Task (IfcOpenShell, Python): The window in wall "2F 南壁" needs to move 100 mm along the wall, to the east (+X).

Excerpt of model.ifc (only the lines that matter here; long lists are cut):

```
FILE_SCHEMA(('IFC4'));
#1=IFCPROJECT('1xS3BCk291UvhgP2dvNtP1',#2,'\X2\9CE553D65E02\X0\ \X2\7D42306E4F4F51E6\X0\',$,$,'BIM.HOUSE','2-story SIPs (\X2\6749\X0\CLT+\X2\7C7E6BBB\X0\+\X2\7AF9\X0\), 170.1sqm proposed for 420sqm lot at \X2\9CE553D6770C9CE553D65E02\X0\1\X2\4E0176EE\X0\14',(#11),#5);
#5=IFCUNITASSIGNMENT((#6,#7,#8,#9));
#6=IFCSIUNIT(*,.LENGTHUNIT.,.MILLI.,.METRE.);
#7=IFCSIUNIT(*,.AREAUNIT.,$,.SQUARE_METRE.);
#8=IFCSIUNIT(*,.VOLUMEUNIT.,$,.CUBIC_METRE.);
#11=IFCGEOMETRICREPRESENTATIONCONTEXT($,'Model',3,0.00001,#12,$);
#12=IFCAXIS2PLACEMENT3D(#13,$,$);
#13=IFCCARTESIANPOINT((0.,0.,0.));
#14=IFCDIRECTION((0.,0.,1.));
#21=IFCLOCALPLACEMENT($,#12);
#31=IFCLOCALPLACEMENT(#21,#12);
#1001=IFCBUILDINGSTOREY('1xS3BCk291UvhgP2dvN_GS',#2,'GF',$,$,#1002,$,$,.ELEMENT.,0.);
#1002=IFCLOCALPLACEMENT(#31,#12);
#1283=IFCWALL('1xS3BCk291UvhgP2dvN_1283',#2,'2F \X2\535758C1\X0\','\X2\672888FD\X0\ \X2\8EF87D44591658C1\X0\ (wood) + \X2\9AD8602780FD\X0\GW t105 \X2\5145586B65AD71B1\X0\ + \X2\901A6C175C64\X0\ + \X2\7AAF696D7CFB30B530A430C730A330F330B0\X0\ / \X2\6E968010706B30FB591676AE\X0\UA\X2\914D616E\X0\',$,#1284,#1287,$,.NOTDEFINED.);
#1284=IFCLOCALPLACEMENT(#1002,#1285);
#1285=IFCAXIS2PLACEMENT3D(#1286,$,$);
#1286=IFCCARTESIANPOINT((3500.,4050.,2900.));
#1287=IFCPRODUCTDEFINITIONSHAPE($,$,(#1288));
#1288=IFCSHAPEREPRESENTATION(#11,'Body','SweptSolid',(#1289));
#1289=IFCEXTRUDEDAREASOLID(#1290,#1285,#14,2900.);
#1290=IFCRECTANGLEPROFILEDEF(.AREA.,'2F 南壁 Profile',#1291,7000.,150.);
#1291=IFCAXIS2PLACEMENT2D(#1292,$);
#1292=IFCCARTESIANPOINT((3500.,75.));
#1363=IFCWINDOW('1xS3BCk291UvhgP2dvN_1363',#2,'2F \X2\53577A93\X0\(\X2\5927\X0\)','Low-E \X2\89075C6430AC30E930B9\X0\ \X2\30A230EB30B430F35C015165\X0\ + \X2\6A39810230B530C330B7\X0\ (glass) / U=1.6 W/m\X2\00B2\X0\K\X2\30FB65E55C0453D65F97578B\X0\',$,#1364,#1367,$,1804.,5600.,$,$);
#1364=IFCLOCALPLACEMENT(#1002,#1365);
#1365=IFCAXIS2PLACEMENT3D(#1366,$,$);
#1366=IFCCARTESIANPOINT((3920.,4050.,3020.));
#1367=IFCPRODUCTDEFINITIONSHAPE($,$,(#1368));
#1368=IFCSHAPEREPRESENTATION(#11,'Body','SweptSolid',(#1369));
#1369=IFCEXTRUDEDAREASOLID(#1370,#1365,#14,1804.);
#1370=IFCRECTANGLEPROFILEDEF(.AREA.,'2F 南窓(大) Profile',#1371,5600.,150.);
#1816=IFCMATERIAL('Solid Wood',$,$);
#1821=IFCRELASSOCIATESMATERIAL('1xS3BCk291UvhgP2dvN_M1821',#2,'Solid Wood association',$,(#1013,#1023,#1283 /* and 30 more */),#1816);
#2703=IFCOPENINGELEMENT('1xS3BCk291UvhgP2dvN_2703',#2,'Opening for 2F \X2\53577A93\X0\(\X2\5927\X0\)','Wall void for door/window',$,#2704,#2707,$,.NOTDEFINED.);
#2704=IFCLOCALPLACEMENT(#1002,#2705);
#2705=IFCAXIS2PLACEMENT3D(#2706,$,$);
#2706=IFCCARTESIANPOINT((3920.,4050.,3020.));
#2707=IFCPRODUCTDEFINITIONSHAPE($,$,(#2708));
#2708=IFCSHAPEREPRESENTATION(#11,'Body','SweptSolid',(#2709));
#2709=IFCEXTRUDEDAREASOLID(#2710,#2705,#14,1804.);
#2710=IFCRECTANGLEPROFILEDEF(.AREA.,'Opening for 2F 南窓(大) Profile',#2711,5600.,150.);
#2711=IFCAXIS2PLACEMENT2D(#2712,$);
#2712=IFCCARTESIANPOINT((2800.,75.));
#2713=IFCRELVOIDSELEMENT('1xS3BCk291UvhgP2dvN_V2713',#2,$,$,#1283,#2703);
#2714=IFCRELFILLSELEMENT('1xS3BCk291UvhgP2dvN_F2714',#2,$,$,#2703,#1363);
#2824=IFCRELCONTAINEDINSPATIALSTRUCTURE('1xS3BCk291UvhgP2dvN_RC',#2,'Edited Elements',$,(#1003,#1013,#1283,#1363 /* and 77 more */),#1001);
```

```python
import ifcopenshell
import ifcopenshell.api.geometry
import ifcopenshell.util.placement
import ifcopenshell.util.unit

model = ifcopenshell.open("model.ifc")
unit_scale = ifcopenshell.util.unit.calculate_unit_scale(model)

window = model.by_guid("1xS3BCk291UvhgP2dvN_1363")
opening = window.FillsVoids[0].RelatingOpeningElement
wall = opening.VoidsElements[0].RelatingBuildingElement

wall_matrix = ifcopenshell.util.placement.get_local_placement(wall.ObjectPlacement)
shift = wall_matrix[:3, 0] * 0.1 / unit_scale
before = ifcopenshell.util.placement.get_local_placement(window.ObjectPlacement)[:3, 3].copy()

# The window is not placed relative to its opening, so move both.
for product in (opening, window):
    matrix = ifcopenshell.util.placement.get_local_placement(product.ObjectPlacement)
    matrix[:3, 3] += shift
    ifcopenshell.api.geometry.edit_object_placement(model, product=product, matrix=matrix, is_si=False)

after = ifcopenshell.util.placement.get_local_placement(window.ObjectPlacement)[:3, 3]
print("window moved by", (after - before).round(3) + 0.0)

model.write("model_edited.ifc")
```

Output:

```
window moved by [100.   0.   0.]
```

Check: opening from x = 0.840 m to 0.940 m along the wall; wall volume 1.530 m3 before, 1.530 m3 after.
